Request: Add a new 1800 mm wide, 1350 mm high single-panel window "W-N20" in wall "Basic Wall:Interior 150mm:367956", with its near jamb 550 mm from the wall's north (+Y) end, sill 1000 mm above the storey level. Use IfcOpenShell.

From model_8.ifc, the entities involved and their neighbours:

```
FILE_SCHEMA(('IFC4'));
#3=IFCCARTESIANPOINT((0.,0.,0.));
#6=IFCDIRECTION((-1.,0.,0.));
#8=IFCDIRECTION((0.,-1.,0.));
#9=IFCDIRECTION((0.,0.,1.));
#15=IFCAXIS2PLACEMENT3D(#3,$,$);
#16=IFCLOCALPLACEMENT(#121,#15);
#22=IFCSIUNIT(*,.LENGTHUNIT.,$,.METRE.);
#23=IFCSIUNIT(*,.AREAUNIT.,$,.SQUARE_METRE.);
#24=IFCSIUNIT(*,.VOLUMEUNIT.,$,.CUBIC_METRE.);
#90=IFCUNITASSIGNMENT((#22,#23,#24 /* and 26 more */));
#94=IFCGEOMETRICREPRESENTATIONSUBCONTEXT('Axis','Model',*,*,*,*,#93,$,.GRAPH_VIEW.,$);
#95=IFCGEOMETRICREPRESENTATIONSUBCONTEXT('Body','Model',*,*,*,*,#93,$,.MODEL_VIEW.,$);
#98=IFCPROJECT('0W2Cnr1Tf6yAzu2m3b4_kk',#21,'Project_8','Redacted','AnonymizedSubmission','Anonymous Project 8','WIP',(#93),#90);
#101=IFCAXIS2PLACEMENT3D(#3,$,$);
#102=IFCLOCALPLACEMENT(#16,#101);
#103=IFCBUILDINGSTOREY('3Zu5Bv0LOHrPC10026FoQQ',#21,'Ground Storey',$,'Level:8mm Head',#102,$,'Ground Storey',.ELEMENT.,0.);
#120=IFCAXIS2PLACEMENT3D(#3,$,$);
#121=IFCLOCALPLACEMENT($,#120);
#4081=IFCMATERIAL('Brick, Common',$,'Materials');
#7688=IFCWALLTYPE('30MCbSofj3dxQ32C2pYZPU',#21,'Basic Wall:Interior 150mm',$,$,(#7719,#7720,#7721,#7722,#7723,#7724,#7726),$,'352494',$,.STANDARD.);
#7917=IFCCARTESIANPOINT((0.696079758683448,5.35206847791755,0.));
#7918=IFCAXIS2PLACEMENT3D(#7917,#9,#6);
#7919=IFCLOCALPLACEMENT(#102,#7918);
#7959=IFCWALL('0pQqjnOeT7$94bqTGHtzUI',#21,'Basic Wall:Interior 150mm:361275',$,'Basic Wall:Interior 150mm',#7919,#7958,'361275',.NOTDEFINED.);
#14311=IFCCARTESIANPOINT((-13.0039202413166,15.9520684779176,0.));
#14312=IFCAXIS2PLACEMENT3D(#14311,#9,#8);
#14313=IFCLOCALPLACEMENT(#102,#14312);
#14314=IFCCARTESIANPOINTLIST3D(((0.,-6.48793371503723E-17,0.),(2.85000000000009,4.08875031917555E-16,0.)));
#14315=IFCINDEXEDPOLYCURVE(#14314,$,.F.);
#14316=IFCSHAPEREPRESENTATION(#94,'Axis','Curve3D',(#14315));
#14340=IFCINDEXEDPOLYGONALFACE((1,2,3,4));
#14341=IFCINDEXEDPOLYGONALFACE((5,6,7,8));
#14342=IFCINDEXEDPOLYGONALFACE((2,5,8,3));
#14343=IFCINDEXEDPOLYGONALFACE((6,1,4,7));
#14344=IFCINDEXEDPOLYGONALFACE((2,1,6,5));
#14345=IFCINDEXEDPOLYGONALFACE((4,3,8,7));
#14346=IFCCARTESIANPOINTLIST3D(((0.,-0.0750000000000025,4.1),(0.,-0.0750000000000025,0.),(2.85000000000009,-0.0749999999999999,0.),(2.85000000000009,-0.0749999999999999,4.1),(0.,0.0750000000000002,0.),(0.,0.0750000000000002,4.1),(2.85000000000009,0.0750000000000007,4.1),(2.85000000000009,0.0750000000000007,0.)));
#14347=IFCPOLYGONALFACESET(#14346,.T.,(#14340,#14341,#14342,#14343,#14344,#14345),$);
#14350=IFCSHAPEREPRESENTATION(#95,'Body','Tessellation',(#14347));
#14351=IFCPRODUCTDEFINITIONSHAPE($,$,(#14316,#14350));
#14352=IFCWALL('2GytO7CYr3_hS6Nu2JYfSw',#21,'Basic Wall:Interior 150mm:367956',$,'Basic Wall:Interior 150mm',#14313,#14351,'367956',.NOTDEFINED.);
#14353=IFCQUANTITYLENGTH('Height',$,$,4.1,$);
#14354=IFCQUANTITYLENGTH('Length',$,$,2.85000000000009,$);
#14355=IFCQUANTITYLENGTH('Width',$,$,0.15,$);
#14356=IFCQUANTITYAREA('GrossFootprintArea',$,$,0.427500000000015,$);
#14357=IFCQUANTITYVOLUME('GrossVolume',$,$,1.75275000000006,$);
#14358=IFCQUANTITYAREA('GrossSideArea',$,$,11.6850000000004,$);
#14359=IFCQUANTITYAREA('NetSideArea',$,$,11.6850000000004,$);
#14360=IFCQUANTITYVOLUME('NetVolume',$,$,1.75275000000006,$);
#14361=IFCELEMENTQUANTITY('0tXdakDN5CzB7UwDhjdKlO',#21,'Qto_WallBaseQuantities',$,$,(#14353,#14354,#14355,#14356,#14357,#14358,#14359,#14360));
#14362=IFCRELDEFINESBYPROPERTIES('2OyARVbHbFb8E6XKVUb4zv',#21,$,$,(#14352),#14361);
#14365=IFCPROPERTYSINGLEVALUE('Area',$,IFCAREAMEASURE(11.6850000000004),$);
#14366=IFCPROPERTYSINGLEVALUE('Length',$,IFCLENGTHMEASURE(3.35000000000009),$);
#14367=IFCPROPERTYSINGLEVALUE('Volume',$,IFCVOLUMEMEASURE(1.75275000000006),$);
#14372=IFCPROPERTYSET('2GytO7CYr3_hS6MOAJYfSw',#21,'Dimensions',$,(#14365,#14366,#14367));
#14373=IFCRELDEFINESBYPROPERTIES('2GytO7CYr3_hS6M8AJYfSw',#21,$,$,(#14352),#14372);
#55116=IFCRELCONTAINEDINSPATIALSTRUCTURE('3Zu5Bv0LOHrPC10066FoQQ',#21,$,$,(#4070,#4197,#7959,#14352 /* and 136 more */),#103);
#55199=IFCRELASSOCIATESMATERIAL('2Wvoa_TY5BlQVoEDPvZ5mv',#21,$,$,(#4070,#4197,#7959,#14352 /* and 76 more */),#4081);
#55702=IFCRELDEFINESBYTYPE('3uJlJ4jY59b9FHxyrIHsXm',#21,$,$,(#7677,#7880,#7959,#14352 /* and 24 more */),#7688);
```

```python
import numpy as np
import ifcopenshell
import ifcopenshell.api.feature
import ifcopenshell.api.geometry
import ifcopenshell.api.pset
import ifcopenshell.api.root
import ifcopenshell.api.spatial
import ifcopenshell.geom
import ifcopenshell.util.element
import ifcopenshell.util.placement
import ifcopenshell.util.representation
import ifcopenshell.util.shape
import ifcopenshell.util.unit

model = ifcopenshell.open("model_8.ifc")
unit_scale = ifcopenshell.util.unit.calculate_unit_scale(model)
area_scale = ifcopenshell.util.unit.calculate_unit_scale(model, "AREAUNIT")
volume_scale = ifcopenshell.util.unit.calculate_unit_scale(model, "VOLUMEUNIT")
settings = ifcopenshell.geom.settings()


def volume(element):
    """Net volume in cubic metres, openings subtracted."""
    shape = ifcopenshell.geom.create_shape(settings, element)
    return ifcopenshell.util.shape.get_volume(shape.geometry)


wall = model.by_id(14352)
storey = ifcopenshell.util.element.get_container(wall, ifc_class="IfcBuildingStorey")
context = ifcopenshell.util.representation.get_context(model, "Model", "Body", "MODEL_VIEW")
before = volume(wall)

width, height, from_end, sill = 1.8, 1.35, 0.55, 1  # metres

# The wall runs along its own X axis, and the end named is its -X end.
wall_shape = ifcopenshell.geom.create_shape(settings, wall)
x, y, z = ifcopenshell.util.shape.get_vertices(wall_shape.geometry).T
start = x.min() + from_end
face, thickness = float(y.min()), float(y.max() - y.min())
wall_matrix = ifcopenshell.util.placement.get_local_placement(wall.ObjectPlacement)
level = ifcopenshell.util.placement.get_local_placement(storey.ObjectPlacement)[2, 3]


def in_wall(x, y):
    """Placement at x, y metres in the wall's axes, at sill height."""
    matrix = wall_matrix.copy()
    matrix[:, 3] = wall_matrix @ np.array([x / unit_scale, y / unit_scale, 0.0, 1.0])
    matrix[2, 3] = level + sill / unit_scale
    return matrix


# Opening: a box that overshoots both wall faces by 50 mm.
opening = ifcopenshell.api.root.create_entity(model, ifc_class="IfcOpeningElement", predefined_type="OPENING")
box = ifcopenshell.api.geometry.add_wall_representation(
    model, context=context, length=width, height=height, thickness=thickness + 0.1
)
ifcopenshell.api.geometry.assign_representation(model, product=opening, representation=box)
ifcopenshell.api.geometry.edit_object_placement(model, product=opening, matrix=in_wall(start, face - 0.05), is_si=False)
ifcopenshell.api.feature.add_feature(model, feature=opening, element=wall)

window = ifcopenshell.api.root.create_entity(model, ifc_class="IfcWindow", name="W-N20", predefined_type="WINDOW")
window.OverallWidth, window.OverallHeight = width / unit_scale, height / unit_scale
window.PartitioningType = "SINGLE_PANEL"
body = ifcopenshell.api.geometry.add_window_representation(
    model,
    context=context,
    overall_width=window.OverallWidth,
    overall_height=window.OverallHeight,
    partition_type="SINGLE_PANEL",
)
ifcopenshell.api.geometry.assign_representation(model, product=window, representation=body)
ifcopenshell.api.spatial.assign_container(model, products=[window], relating_structure=storey)
ifcopenshell.api.feature.add_filling(model, opening=opening, element=window)

# Centre the window in the wall's thickness.
ifcopenshell.api.geometry.edit_object_placement(model, product=window, matrix=in_wall(start, face), is_si=False)
window_shape = ifcopenshell.geom.create_shape(settings, window)
depth = ifcopenshell.util.shape.get_vertices(window_shape.geometry)[:, 1]
offset = face + thickness / 2 - (depth.min() + depth.max()) / 2
ifcopenshell.api.geometry.edit_object_placement(model, product=window, matrix=in_wall(start, offset), is_si=False)

after = volume(wall)

# Update the wall's stored quantities.
qto = model.by_id(ifcopenshell.util.element.get_pset(wall, "Qto_WallBaseQuantities", should_inherit=False)["id"])
ifcopenshell.api.pset.edit_qto(model, qto=qto, properties={
    "NetSideArea": after / thickness / area_scale,
    "NetVolume": after / volume_scale,
})
pset = model.by_id(ifcopenshell.util.element.get_pset(wall, "Dimensions", should_inherit=False)["id"])
ifcopenshell.api.pset.edit_pset(model, pset=pset, properties={
    "Area": model.create_entity("IfcAreaMeasure", after / thickness / area_scale),
    "Volume": model.create_entity("IfcVolumeMeasure", after / volume_scale),
})

print(f"wall volume {before:.3f} -> {after:.3f} m3")

model.write("model_8_edited.ifc")
```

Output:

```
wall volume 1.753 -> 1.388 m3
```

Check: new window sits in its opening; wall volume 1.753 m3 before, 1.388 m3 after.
